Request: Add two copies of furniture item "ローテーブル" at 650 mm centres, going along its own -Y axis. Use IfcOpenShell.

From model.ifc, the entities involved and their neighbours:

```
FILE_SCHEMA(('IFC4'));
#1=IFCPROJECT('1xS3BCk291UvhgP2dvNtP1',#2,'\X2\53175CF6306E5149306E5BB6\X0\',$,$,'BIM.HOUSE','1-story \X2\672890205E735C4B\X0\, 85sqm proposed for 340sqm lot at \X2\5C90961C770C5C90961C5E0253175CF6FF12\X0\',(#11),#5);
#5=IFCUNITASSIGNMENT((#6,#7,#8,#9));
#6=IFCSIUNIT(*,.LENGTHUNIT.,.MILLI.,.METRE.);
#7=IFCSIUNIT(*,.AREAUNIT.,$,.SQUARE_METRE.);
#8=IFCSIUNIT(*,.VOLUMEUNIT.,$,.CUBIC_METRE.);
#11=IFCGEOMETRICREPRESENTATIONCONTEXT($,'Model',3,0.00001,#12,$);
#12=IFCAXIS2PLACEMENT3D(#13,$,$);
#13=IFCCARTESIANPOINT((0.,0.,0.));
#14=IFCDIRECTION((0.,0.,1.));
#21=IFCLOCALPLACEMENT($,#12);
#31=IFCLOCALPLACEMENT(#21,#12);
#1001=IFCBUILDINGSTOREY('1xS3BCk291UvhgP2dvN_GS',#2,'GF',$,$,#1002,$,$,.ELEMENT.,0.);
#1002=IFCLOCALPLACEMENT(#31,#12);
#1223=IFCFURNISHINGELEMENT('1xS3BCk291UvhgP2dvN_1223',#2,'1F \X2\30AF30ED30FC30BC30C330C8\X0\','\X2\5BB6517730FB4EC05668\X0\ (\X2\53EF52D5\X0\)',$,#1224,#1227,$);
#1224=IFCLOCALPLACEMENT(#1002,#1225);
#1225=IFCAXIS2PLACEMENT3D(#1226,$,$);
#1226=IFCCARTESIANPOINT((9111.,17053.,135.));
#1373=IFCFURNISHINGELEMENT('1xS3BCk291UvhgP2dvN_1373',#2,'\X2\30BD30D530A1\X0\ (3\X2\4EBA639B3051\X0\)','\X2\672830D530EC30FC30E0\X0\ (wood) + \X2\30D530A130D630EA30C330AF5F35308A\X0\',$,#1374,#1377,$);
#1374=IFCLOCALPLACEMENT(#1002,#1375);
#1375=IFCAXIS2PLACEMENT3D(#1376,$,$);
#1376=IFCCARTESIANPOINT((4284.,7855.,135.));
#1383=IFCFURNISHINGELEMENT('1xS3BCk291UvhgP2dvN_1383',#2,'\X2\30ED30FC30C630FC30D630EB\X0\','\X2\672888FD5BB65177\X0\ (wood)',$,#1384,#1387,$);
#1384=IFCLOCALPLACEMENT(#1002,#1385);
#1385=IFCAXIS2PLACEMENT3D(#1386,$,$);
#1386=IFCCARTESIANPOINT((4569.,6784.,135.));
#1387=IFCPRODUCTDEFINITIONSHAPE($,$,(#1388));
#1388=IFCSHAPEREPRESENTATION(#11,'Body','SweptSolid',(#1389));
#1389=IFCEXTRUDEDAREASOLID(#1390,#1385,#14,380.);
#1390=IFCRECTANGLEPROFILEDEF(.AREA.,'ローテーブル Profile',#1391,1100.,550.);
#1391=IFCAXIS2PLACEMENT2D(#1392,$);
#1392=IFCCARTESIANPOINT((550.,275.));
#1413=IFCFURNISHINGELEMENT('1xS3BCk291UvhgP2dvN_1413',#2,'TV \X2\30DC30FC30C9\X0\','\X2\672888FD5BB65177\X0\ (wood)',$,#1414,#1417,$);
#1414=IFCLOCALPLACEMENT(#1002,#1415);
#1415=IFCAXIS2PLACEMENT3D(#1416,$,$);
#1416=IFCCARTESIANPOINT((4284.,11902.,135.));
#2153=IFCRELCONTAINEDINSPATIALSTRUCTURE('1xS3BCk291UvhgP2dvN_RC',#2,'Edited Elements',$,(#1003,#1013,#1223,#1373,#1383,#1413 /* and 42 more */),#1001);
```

```python
import ifcopenshell
import ifcopenshell.api.geometry
import ifcopenshell.api.root
import ifcopenshell.util.element
import ifcopenshell.util.placement
import ifcopenshell.util.unit

model = ifcopenshell.open("model.ifc")
unit_scale = ifcopenshell.util.unit.calculate_unit_scale(model)


def reuse_history(source, copy):
    """copy_class also copies each property set's owner history, people and application; keep the originals."""
    for rel in copy.IsDefinedBy:
        if rel.is_a("IfcRelDefinesByProperties") and (history := rel.RelatingPropertyDefinition.OwnerHistory):
            rel.RelatingPropertyDefinition.OwnerHistory = source.OwnerHistory
            ifcopenshell.util.element.remove_deep2(model, history)


source = model.by_guid("1xS3BCk291UvhgP2dvN_1383")
base = ifcopenshell.util.placement.get_local_placement(source.ObjectPlacement)
step = -base[:3, 1] * 0.65 / unit_scale

for i in range(1, 3):
    copy = ifcopenshell.api.root.copy_class(model, product=source)
    copy.Representation = ifcopenshell.util.element.copy_deep(
        model, source.Representation, exclude=["IfcGeometricRepresentationContext", "IfcRepresentationMap"]
    )
    reuse_history(source, copy)
    matrix = base.copy()
    matrix[:3, 3] += i * step
    print("added at", matrix[:3, 3].round(3) + 0.0)
    ifcopenshell.api.geometry.edit_object_placement(model, product=copy, matrix=matrix, is_si=False)

model.write("model_edited.ifc")
```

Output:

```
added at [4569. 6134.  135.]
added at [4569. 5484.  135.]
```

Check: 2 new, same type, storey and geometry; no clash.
